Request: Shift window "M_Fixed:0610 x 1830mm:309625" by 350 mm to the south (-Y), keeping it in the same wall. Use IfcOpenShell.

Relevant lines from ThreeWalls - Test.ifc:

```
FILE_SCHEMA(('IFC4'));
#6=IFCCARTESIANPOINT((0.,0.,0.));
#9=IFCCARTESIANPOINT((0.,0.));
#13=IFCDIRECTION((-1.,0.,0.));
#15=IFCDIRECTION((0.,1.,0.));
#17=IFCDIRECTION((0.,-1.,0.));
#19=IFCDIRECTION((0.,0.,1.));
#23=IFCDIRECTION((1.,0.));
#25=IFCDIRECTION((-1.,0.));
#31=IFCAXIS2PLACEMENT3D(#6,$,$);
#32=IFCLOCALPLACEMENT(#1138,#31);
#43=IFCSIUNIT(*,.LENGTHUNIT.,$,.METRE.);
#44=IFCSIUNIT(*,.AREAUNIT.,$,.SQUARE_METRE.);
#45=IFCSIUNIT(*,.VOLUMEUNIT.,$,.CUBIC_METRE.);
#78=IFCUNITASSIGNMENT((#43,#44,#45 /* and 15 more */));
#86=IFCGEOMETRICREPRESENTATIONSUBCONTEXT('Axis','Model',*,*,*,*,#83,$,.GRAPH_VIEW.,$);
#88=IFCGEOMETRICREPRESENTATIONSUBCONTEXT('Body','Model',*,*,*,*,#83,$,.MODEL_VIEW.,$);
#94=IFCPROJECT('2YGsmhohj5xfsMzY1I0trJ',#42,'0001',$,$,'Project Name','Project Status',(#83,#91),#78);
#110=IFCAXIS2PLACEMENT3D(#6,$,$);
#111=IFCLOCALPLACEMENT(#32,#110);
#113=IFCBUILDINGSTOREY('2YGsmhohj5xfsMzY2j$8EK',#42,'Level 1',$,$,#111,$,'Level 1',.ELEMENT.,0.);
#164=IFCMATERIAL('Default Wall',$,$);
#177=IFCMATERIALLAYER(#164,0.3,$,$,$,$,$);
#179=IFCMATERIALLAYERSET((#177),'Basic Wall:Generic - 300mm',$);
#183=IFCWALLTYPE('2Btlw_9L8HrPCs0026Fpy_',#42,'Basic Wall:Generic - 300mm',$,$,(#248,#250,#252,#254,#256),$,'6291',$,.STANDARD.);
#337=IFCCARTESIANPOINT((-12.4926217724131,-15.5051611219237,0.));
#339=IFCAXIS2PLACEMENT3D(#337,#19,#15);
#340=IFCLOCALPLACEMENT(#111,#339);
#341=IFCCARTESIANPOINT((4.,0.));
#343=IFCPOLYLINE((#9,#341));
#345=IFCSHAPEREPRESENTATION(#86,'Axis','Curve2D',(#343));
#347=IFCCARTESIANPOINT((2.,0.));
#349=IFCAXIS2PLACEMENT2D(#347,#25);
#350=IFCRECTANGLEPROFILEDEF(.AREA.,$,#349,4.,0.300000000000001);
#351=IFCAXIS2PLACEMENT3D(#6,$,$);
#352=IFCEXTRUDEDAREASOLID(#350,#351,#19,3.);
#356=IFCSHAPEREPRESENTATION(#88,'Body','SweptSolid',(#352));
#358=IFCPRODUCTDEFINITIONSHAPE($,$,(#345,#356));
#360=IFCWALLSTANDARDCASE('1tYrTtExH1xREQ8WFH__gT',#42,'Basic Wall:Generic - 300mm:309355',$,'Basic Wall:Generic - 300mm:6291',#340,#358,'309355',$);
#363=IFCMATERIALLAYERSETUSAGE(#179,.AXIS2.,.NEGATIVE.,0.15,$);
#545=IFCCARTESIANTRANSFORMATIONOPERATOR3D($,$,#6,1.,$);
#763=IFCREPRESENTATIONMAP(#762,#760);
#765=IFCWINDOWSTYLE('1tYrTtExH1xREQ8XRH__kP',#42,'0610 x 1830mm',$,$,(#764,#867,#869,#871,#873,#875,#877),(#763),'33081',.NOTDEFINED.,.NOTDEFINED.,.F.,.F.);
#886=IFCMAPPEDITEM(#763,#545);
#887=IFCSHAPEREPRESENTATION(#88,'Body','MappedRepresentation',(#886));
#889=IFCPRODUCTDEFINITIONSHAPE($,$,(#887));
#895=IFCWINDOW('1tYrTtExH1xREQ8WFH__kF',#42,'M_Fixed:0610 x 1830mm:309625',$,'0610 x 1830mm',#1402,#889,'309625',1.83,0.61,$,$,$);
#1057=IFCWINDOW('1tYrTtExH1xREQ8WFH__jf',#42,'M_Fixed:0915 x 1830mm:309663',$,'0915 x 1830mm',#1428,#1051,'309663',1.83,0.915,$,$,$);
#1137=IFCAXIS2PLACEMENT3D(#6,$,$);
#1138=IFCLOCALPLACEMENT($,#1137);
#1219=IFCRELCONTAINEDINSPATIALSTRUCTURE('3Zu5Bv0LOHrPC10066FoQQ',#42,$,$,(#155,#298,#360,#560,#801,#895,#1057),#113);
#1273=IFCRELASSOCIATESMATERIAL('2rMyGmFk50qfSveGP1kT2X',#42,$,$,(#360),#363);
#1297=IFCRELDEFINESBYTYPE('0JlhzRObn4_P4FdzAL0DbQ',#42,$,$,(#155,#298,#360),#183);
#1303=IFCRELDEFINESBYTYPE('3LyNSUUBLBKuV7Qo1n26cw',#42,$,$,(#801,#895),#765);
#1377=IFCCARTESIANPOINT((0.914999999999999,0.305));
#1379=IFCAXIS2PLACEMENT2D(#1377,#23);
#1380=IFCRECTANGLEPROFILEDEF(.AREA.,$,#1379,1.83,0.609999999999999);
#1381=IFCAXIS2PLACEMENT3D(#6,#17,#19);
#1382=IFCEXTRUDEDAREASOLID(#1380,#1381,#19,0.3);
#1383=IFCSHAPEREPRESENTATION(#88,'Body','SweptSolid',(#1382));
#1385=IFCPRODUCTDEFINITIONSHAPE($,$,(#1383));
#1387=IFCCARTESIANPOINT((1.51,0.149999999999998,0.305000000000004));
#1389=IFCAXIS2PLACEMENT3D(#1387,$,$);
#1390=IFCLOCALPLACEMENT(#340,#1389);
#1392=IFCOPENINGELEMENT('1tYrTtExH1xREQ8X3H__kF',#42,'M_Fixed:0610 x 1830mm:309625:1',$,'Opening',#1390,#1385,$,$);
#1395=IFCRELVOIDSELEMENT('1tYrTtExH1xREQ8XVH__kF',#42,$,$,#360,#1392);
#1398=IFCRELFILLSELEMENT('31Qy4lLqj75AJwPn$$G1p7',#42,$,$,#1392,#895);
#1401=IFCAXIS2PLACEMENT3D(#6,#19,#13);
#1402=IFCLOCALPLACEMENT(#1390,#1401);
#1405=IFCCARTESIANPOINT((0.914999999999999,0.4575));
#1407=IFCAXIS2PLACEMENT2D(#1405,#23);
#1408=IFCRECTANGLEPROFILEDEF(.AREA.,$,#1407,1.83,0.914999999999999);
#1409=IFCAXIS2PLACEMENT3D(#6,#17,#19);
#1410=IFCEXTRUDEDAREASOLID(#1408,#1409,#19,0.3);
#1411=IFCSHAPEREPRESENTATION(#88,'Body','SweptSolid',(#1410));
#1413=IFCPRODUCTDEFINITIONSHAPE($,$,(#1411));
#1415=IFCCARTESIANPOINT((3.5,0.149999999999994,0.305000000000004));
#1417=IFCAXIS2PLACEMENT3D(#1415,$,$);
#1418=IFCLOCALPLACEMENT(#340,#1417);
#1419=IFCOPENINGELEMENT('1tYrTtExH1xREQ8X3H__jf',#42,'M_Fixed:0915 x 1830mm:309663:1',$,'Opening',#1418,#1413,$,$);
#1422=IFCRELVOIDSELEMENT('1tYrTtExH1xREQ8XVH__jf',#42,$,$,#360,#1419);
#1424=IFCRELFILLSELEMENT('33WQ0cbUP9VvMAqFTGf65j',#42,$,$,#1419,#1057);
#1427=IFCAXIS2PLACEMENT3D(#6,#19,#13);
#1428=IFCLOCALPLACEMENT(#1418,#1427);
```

```python
import ifcopenshell
import ifcopenshell.api.geometry
import ifcopenshell.util.placement

model = ifcopenshell.open("ThreeWalls - Test.ifc")

window = model.by_id(895)
opening = window.FillsVoids[0].RelatingOpeningElement
wall = opening.VoidsElements[0].RelatingBuildingElement

wall_matrix = ifcopenshell.util.placement.get_local_placement(wall.ObjectPlacement)
shift = wall_matrix[:3, 0] * -0.35
before = ifcopenshell.util.placement.get_local_placement(window.ObjectPlacement)[:3, 3].copy()

# The window is placed relative to its opening, so it follows when the opening moves.
matrix = ifcopenshell.util.placement.get_local_placement(opening.ObjectPlacement)
matrix[:3, 3] += shift
ifcopenshell.api.geometry.edit_object_placement(
    model, product=opening, matrix=matrix, is_si=False, should_transform_children=True
)

after = ifcopenshell.util.placement.get_local_placement(window.ObjectPlacement)[:3, 3]
print("window moved by", (after - before).round(3) + 0.0)

model.write("ThreeWalls - Test_rev.ifc")
```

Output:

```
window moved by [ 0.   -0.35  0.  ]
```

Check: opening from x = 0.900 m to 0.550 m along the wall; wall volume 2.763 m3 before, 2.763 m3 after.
